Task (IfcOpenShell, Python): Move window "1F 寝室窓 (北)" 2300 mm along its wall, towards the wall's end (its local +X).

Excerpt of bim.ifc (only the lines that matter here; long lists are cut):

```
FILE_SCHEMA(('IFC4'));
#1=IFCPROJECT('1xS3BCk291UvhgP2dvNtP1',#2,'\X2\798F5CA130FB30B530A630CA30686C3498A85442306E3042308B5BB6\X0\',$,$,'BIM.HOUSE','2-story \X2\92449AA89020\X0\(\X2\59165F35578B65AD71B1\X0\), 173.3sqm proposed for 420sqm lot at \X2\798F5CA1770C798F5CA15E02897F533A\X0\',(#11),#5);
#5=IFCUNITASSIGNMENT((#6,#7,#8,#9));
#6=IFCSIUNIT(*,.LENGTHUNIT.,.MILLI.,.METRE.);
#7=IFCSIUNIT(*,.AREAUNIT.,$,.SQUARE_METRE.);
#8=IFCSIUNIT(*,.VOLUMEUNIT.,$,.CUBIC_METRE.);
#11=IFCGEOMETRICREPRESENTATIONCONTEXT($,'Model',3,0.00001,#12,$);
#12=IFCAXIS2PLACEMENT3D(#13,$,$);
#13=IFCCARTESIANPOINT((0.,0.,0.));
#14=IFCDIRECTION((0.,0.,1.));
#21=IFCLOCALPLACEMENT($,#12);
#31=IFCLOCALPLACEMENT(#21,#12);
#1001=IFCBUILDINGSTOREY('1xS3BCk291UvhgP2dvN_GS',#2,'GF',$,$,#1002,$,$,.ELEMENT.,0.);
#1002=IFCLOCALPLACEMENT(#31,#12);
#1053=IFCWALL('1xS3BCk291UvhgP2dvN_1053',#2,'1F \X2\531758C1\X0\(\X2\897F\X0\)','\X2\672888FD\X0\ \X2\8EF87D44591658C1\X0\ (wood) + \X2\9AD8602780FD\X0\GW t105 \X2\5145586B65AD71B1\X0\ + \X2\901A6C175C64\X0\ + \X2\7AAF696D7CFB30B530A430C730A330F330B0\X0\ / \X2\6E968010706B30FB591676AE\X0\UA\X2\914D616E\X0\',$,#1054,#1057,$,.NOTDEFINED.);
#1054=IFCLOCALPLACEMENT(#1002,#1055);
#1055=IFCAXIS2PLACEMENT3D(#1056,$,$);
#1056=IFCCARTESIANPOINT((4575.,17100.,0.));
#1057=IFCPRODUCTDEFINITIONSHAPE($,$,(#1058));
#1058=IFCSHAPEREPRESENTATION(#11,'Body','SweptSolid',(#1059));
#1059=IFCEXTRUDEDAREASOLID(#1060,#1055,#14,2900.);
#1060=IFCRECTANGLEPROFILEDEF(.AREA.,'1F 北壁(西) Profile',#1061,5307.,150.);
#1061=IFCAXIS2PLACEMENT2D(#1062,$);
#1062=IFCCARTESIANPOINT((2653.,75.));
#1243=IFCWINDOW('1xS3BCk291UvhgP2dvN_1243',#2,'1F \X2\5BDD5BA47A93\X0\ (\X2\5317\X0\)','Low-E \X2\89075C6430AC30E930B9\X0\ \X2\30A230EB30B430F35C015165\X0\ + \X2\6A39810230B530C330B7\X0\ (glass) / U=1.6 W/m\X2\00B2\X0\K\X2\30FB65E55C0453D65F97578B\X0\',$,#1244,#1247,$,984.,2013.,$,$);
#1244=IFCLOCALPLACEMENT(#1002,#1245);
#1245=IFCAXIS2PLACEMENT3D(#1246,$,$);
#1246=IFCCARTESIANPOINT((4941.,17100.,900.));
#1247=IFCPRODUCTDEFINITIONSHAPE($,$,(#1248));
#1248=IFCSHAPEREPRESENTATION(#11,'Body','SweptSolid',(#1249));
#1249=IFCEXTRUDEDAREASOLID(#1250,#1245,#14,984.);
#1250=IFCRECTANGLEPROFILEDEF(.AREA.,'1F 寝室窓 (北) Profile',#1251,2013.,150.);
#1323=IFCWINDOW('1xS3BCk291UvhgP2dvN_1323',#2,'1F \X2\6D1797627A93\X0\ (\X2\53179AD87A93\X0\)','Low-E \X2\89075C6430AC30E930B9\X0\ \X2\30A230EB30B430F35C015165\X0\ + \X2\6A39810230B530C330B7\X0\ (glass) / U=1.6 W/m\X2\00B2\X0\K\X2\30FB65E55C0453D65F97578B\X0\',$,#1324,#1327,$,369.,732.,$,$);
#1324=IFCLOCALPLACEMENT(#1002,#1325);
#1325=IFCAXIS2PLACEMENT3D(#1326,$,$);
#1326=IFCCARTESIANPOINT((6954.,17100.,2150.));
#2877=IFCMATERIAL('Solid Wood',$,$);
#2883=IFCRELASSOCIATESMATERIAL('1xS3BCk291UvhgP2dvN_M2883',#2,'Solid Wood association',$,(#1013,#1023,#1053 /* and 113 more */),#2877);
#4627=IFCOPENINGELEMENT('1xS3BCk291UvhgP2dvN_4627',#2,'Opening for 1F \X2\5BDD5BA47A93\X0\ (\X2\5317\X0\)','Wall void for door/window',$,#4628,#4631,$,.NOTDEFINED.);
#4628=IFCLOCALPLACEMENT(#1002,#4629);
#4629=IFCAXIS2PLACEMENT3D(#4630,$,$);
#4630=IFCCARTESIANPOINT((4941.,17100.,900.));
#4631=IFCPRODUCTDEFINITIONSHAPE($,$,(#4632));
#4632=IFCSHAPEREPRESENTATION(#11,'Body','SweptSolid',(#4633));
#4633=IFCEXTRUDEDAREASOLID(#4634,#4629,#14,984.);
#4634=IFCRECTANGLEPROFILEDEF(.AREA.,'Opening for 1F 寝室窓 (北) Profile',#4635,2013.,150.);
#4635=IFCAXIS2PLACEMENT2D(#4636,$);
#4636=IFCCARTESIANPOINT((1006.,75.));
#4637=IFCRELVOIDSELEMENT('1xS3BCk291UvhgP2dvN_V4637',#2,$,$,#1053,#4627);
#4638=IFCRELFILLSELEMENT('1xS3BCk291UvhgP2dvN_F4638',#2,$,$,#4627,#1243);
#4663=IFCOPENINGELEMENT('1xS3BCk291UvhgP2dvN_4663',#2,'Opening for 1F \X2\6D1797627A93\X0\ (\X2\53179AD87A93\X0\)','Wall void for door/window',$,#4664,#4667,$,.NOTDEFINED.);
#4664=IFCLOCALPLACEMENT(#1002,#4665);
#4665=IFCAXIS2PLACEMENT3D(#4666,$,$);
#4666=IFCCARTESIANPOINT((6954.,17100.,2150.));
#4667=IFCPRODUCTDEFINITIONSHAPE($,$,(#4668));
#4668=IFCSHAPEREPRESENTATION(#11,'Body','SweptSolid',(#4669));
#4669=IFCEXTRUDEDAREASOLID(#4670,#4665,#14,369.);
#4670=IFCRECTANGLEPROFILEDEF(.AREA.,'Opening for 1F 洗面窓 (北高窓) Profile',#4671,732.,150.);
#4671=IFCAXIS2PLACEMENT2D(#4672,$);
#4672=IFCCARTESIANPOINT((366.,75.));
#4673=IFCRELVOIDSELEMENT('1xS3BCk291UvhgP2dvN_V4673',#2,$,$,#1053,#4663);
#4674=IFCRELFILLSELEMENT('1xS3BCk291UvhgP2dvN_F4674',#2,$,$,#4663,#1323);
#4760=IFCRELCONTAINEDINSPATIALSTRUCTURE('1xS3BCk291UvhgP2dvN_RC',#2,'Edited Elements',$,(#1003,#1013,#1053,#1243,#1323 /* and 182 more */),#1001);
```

```python
import ifcopenshell
import ifcopenshell.api.geometry
import ifcopenshell.util.placement
import ifcopenshell.util.unit

model = ifcopenshell.open("bim.ifc")
unit_scale = ifcopenshell.util.unit.calculate_unit_scale(model)

window = model.by_guid("1xS3BCk291UvhgP2dvN_1243")
opening = window.FillsVoids[0].RelatingOpeningElement
wall = opening.VoidsElements[0].RelatingBuildingElement

wall_matrix = ifcopenshell.util.placement.get_local_placement(wall.ObjectPlacement)
shift = wall_matrix[:3, 0] * 2.3 / unit_scale
before = ifcopenshell.util.placement.get_local_placement(window.ObjectPlacement)[:3, 3].copy()

# The window is not placed relative to its opening, so move both.
for product in (opening, window):
    matrix = ifcopenshell.util.placement.get_local_placement(product.ObjectPlacement)
    matrix[:3, 3] += shift
    ifcopenshell.api.geometry.edit_object_placement(model, product=product, matrix=matrix, is_si=False)

after = ifcopenshell.util.placement.get_local_placement(window.ObjectPlacement)[:3, 3]
print("window moved by", (after - before).round(3) + 0.0)

model.write("bim_updated.ifc")
```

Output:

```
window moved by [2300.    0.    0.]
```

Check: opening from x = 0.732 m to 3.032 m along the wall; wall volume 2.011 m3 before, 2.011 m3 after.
